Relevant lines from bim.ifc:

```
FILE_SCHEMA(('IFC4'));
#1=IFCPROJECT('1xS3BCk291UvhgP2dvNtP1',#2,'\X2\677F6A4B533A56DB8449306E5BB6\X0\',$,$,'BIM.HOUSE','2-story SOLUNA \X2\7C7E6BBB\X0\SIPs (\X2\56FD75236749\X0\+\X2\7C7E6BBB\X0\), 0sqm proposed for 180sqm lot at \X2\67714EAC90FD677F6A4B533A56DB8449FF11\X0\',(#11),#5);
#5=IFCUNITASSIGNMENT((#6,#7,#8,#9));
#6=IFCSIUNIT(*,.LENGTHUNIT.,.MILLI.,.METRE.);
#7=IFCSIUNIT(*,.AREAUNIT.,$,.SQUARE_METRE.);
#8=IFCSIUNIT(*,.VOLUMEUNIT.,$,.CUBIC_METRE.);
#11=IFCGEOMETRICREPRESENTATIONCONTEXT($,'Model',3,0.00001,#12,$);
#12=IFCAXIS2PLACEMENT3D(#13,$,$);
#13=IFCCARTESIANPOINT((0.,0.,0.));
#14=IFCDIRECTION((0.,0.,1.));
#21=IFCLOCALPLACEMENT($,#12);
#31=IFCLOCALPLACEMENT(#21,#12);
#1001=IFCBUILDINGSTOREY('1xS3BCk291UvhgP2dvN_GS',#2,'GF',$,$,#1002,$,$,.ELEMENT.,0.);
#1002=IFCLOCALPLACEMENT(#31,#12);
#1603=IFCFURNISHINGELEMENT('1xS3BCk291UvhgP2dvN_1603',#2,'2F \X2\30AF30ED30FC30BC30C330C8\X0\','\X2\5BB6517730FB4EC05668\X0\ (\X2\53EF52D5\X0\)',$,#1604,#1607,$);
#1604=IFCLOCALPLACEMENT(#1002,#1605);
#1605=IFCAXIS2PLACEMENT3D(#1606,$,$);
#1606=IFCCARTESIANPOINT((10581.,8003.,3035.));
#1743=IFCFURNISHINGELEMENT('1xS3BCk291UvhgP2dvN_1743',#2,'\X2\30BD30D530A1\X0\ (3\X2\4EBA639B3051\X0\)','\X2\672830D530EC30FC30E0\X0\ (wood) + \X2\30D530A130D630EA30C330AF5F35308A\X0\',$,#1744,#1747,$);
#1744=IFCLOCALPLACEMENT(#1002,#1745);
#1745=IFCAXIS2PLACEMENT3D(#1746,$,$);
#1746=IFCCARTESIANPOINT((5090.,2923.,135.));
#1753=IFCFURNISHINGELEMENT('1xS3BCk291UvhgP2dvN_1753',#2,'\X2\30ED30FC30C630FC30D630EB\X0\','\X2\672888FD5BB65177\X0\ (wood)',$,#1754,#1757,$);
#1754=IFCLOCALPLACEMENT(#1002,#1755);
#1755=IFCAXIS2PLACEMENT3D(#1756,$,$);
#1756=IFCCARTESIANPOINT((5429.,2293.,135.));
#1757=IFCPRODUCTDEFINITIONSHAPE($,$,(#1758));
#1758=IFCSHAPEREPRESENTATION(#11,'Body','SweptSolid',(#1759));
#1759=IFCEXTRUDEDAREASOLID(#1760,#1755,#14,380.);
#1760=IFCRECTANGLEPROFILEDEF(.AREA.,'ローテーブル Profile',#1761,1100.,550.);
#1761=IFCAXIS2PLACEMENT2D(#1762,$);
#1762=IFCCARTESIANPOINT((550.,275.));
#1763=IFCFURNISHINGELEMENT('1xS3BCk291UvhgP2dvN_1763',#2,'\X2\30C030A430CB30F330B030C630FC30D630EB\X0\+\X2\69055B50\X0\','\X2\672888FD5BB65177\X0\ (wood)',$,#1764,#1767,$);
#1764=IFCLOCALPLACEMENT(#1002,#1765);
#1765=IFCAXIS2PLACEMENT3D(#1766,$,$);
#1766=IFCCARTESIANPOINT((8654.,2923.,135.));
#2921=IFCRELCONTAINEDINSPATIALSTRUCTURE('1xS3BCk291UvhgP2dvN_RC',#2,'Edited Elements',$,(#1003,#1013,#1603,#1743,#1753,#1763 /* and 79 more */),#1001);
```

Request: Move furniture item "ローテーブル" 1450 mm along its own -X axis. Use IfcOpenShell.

```python
import ifcopenshell
import ifcopenshell.api.geometry
import ifcopenshell.util.placement
import ifcopenshell.util.unit

model = ifcopenshell.open("bim.ifc")
unit_scale = ifcopenshell.util.unit.calculate_unit_scale(model)

item = model.by_guid("1xS3BCk291UvhgP2dvN_1753")
matrix = ifcopenshell.util.placement.get_local_placement(item.ObjectPlacement)
matrix[:3, 3] -= matrix[:3, 0] * 1.45 / unit_scale
ifcopenshell.api.geometry.edit_object_placement(model, product=item, matrix=matrix, is_si=False)

print(ifcopenshell.util.placement.get_local_placement(item.ObjectPlacement).round(3) + 0.0)

model.write("bim_v2.ifc")
```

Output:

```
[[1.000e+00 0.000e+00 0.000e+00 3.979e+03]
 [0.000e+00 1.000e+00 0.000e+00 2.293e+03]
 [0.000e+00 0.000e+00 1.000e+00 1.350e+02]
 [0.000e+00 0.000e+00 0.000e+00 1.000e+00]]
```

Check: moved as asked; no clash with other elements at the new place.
